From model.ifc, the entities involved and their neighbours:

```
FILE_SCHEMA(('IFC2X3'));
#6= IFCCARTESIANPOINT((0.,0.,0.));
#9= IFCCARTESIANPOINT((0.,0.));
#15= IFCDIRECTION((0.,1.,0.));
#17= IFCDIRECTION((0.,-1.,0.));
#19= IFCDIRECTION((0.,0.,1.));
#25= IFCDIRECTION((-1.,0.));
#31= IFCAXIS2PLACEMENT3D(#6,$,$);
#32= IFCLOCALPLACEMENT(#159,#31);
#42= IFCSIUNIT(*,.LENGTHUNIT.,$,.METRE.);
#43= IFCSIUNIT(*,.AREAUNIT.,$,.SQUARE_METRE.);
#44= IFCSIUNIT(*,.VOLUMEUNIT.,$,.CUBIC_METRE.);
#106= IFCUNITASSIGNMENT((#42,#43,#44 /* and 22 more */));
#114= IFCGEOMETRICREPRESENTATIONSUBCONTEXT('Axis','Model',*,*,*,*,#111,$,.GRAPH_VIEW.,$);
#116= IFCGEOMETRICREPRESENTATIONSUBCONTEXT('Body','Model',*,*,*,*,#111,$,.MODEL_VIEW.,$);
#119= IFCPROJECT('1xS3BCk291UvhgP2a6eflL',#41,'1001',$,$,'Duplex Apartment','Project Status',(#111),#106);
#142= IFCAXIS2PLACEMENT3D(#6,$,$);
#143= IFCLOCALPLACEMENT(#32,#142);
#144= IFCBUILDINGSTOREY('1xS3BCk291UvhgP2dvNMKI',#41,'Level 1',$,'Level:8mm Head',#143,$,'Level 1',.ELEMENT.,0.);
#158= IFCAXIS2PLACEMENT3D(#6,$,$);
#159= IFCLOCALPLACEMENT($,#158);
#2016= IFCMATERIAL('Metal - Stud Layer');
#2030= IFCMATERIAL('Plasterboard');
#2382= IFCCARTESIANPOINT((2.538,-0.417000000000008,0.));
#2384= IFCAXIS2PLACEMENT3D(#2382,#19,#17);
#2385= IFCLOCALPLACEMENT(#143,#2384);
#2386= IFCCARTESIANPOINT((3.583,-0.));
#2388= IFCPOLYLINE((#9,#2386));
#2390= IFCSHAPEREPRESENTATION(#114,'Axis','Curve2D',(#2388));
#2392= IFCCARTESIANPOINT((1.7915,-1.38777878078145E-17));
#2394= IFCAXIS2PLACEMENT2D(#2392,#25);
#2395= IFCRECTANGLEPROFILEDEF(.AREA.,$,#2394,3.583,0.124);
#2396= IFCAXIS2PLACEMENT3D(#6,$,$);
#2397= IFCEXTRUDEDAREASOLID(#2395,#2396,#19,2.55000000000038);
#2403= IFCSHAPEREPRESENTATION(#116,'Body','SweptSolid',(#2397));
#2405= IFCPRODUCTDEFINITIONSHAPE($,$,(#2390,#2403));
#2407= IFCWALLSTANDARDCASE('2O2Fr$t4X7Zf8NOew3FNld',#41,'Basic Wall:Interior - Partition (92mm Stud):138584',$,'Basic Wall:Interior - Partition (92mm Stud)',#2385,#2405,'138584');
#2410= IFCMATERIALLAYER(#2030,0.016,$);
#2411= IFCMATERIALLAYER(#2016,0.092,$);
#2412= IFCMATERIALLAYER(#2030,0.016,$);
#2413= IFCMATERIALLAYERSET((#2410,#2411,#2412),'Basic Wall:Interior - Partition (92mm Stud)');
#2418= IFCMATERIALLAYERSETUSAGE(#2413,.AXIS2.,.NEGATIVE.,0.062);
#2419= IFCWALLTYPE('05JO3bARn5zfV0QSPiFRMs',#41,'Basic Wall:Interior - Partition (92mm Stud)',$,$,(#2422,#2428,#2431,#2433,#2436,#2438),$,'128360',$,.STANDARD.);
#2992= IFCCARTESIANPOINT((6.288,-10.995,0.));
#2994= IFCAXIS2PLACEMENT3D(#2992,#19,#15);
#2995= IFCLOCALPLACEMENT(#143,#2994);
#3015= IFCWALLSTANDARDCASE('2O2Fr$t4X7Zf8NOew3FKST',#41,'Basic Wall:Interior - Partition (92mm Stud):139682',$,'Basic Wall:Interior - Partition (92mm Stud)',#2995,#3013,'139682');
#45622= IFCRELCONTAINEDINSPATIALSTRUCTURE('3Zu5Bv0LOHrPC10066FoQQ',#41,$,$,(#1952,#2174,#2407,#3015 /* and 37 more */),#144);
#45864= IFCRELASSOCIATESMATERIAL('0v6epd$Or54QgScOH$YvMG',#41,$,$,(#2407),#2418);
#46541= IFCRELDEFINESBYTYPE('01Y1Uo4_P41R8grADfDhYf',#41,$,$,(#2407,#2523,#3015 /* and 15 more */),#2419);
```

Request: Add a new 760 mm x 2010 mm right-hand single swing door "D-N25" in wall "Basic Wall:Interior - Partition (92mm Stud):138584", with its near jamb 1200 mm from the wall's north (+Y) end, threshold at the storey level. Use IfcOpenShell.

```python
import numpy as np
import ifcopenshell
import ifcopenshell.api.feature
import ifcopenshell.api.geometry
import ifcopenshell.api.root
import ifcopenshell.api.spatial
import ifcopenshell.api.type
import ifcopenshell.geom
import ifcopenshell.util.element
import ifcopenshell.util.placement
import ifcopenshell.util.representation
import ifcopenshell.util.shape
import ifcopenshell.util.unit

model = ifcopenshell.open("model.ifc")
unit_scale = ifcopenshell.util.unit.calculate_unit_scale(model)
settings = ifcopenshell.geom.settings()


def volume(element):
    """Net volume in cubic metres, openings subtracted."""
    shape = ifcopenshell.geom.create_shape(settings, element)
    return ifcopenshell.util.shape.get_volume(shape.geometry)


wall = model.by_id(2407)
storey = ifcopenshell.util.element.get_container(wall, ifc_class="IfcBuildingStorey")
context = ifcopenshell.util.representation.get_context(model, "Model", "Body", "MODEL_VIEW")
before = volume(wall)

width, height, from_end, sill = 0.76, 2.01, 1.2, 0.0  # metres

# The wall runs along its own X axis, and the end named is its -X end.
wall_shape = ifcopenshell.geom.create_shape(settings, wall)
x, y, z = ifcopenshell.util.shape.get_vertices(wall_shape.geometry).T
start = x.min() + from_end
face, thickness = float(y.min()), float(y.max() - y.min())
wall_matrix = ifcopenshell.util.placement.get_local_placement(wall.ObjectPlacement)
level = ifcopenshell.util.placement.get_local_placement(storey.ObjectPlacement)[2, 3]


def in_wall(x, y):
    """Placement at x, y metres in the wall's axes, at sill height."""
    matrix = wall_matrix.copy()
    matrix[:, 3] = wall_matrix @ np.array([x / unit_scale, y / unit_scale, 0.0, 1.0])
    matrix[2, 3] = level + sill / unit_scale
    return matrix


# Opening: a box that overshoots both wall faces by 50 mm.
opening = ifcopenshell.api.root.create_entity(model, ifc_class="IfcOpeningElement")
box = ifcopenshell.api.geometry.add_wall_representation(
    model, context=context, length=width, height=height, thickness=thickness + 0.1
)
ifcopenshell.api.geometry.assign_representation(model, product=opening, representation=box)
ifcopenshell.api.geometry.edit_object_placement(model, product=opening, matrix=in_wall(start, face - 0.05), is_si=False)
ifcopenshell.api.feature.add_feature(model, feature=opening, element=wall)

door = ifcopenshell.api.root.create_entity(model, ifc_class="IfcDoor", name="D-N25")
door.OverallWidth, door.OverallHeight = width / unit_scale, height / unit_scale
body = ifcopenshell.api.geometry.add_door_representation(
    model,
    context=context,
    overall_width=door.OverallWidth,
    overall_height=door.OverallHeight,
    operation_type="SINGLE_SWING_RIGHT",
    lining_properties={"LiningDepth": thickness / unit_scale, "ThresholdDepth": thickness / unit_scale},
)
ifcopenshell.api.geometry.assign_representation(model, product=door, representation=body)
ifcopenshell.api.spatial.assign_container(model, products=[door], relating_structure=storey)
fills = ifcopenshell.api.feature.add_filling(model, opening=opening, element=door)
fills.OwnerHistory = door.OwnerHistory  # required in IFC2X3

# IFC2X3 keeps the operation on the door style.
style = ifcopenshell.api.root.create_entity(model, ifc_class="IfcDoorStyle", name="D-N25")
style.OperationType, style.ConstructionType = "SINGLE_SWING_RIGHT", "NOTDEFINED"
style.ParameterTakesPrecedence = style.Sizeable = False
ifcopenshell.api.type.assign_type(model, related_objects=[door], relating_type=style)

# The lining spans the wall, so the door starts at the wall face.
ifcopenshell.api.geometry.edit_object_placement(model, product=door, matrix=in_wall(start, face), is_si=False)

after = volume(wall)

print(f"wall volume {before:.3f} -> {after:.3f} m3")

model.write("model_updated.ifc")
```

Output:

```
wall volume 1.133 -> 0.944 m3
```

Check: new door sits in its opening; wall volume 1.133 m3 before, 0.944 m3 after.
